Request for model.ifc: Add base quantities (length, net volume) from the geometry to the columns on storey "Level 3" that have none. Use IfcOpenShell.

First a look at what the model holds.

```python
import ifcopenshell
import ifcopenshell.util.element
import ifcopenshell.util.unit

model = ifcopenshell.open("model.ifc")
print(model.schema)
for unit_type in ("LENGTHUNIT", "AREAUNIT", "VOLUMEUNIT"):
    print(unit_type, ifcopenshell.util.unit.calculate_unit_scale(model, unit_type))
storey = next(s for s in model.by_type("IfcBuildingStorey") if s.Name == "Level 3")
columns = [e for e in ifcopenshell.util.element.get_decomposition(storey) if e.is_a("IfcColumn")]
for e in sorted(columns, key=lambda e: e.id()):
    print(e.id(), e.is_a(), e.Name, list(ifcopenshell.util.element.get_psets(e, qtos_only=True)), sep=" | ")
```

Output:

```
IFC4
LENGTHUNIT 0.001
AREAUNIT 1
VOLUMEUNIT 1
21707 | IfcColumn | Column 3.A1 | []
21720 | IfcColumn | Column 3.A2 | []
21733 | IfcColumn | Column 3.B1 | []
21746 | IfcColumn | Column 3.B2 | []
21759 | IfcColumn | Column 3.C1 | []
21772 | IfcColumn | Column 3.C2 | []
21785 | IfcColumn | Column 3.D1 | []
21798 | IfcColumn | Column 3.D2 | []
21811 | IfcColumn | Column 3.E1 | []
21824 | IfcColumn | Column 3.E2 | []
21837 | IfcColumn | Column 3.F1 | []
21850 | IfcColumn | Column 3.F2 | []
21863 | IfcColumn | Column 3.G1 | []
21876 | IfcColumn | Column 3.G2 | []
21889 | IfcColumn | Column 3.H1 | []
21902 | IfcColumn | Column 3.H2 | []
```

```python
import ifcopenshell
import ifcopenshell.api.pset
import ifcopenshell.geom
import ifcopenshell.util.element
import ifcopenshell.util.shape
import ifcopenshell.util.unit

model = ifcopenshell.open("model.ifc")
unit_scale = ifcopenshell.util.unit.calculate_unit_scale(model)
volume_scale = ifcopenshell.util.unit.calculate_unit_scale(model, "VOLUMEUNIT")
settings = ifcopenshell.geom.settings()

storey = next(s for s in model.by_type("IfcBuildingStorey") if s.Name == "Level 3")
columns = [e for e in ifcopenshell.util.element.get_decomposition(storey) if e.is_a("IfcColumn")]

for e in sorted(columns, key=lambda e: e.id()):
    if ifcopenshell.util.element.get_psets(e, qtos_only=True, should_inherit=False):
        continue
    # Geometry comes back in metres, in the element's own axes.
    shape = ifcopenshell.geom.create_shape(settings, e)
    values = {
        "Length": ifcopenshell.util.shape.get_z(shape.geometry) / unit_scale,
        "NetVolume": ifcopenshell.util.shape.get_volume(shape.geometry) / volume_scale,
    }
    qto = ifcopenshell.api.pset.add_qto(model, product=e, name="Qto_ColumnBaseQuantities")
    ifcopenshell.api.pset.edit_qto(model, qto=qto, properties=values)
    print(e.id(), {k: round(v, 3) for k, v in values.items()})

model.write("model_v2.ifc")
```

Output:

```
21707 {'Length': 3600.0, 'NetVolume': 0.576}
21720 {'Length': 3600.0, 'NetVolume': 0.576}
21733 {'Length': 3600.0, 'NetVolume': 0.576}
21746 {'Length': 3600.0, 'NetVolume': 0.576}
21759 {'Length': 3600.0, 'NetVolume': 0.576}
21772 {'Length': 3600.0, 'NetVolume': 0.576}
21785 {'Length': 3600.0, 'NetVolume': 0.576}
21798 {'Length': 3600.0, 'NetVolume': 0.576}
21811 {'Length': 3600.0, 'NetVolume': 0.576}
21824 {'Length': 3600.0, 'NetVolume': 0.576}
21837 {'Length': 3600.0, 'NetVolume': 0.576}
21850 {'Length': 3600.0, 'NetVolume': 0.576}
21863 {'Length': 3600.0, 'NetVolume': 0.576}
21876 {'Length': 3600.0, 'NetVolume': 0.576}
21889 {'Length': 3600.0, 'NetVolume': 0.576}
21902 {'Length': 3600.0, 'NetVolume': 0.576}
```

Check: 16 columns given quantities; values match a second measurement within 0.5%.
